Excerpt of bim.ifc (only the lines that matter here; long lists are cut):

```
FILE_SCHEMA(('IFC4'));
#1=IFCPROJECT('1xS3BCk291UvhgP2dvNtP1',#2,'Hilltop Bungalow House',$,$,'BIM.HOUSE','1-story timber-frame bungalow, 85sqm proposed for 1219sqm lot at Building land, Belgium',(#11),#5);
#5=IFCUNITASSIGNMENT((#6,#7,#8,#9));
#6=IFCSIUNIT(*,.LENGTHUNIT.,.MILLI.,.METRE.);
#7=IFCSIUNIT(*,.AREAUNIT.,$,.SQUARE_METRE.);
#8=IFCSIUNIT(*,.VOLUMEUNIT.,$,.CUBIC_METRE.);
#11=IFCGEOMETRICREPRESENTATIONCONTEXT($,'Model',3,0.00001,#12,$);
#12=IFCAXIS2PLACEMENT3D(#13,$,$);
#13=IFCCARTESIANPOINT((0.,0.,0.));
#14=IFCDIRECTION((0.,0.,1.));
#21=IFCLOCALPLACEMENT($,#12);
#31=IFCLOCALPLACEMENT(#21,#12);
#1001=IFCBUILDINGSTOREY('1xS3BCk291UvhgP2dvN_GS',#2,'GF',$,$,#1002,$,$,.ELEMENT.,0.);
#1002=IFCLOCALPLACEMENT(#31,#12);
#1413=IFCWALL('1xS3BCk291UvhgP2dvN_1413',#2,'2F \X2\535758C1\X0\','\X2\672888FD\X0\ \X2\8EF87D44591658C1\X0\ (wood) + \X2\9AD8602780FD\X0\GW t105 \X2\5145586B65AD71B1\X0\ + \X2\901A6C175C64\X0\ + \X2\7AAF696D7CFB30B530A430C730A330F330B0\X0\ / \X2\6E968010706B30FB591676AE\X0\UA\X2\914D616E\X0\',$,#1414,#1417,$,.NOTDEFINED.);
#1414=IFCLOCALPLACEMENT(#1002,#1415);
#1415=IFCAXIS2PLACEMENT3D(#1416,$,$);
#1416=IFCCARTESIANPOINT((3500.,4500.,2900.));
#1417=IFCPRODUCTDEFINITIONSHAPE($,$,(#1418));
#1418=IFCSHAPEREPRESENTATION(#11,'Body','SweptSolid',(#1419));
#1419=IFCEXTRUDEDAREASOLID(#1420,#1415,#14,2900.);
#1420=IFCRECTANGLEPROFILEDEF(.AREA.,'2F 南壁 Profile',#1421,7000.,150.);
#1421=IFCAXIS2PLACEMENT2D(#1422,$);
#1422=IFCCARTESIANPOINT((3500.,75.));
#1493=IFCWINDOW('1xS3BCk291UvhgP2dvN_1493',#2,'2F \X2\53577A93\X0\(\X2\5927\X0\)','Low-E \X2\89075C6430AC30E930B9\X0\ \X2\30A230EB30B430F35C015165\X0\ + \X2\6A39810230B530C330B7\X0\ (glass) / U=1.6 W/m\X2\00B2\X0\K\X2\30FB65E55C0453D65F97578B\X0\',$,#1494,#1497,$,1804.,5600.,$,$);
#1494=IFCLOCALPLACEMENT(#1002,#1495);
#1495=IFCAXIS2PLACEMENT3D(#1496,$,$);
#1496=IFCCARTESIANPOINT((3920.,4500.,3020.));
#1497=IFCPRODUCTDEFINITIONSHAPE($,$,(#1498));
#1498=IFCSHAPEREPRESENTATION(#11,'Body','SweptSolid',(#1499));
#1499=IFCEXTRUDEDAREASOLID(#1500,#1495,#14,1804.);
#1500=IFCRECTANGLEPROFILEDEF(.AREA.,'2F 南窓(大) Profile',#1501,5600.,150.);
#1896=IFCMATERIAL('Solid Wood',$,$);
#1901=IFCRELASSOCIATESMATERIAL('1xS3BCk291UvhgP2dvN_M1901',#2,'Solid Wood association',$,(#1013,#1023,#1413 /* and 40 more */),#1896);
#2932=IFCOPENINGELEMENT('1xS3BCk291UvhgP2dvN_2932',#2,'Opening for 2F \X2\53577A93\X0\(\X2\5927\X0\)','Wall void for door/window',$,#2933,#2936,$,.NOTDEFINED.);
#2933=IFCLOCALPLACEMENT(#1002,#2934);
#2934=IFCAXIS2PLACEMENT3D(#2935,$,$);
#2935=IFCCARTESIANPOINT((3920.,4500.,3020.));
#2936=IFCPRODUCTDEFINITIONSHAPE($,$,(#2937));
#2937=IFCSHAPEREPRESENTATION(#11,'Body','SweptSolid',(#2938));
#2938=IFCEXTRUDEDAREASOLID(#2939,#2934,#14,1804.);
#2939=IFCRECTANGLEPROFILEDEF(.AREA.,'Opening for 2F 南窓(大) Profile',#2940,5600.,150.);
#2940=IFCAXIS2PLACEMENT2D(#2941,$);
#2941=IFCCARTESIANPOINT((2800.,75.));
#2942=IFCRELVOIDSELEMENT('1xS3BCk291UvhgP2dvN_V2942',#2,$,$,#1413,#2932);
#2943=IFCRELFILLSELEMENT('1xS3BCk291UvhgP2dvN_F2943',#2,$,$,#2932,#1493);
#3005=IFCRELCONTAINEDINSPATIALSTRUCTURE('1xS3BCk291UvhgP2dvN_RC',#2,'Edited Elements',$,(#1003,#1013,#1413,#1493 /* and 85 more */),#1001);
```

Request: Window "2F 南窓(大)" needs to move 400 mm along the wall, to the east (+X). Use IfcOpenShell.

```python
import ifcopenshell
import ifcopenshell.api.geometry
import ifcopenshell.util.placement
import ifcopenshell.util.unit

model = ifcopenshell.open("bim.ifc")
unit_scale = ifcopenshell.util.unit.calculate_unit_scale(model)

window = model.by_guid("1xS3BCk291UvhgP2dvN_1493")
opening = window.FillsVoids[0].RelatingOpeningElement
wall = opening.VoidsElements[0].RelatingBuildingElement

wall_matrix = ifcopenshell.util.placement.get_local_placement(wall.ObjectPlacement)
shift = wall_matrix[:3, 0] * 0.4 / unit_scale
before = ifcopenshell.util.placement.get_local_placement(window.ObjectPlacement)[:3, 3].copy()

# The window is not placed relative to its opening, so move both.
for product in (opening, window):
    matrix = ifcopenshell.util.placement.get_local_placement(product.ObjectPlacement)
    matrix[:3, 3] += shift
    ifcopenshell.api.geometry.edit_object_placement(model, product=product, matrix=matrix, is_si=False)

after = ifcopenshell.util.placement.get_local_placement(window.ObjectPlacement)[:3, 3]
print("window moved by", (after - before).round(3) + 0.0)

model.write("bim_updated.ifc")
```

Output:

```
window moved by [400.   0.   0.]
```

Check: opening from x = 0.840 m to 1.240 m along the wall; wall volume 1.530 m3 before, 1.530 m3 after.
